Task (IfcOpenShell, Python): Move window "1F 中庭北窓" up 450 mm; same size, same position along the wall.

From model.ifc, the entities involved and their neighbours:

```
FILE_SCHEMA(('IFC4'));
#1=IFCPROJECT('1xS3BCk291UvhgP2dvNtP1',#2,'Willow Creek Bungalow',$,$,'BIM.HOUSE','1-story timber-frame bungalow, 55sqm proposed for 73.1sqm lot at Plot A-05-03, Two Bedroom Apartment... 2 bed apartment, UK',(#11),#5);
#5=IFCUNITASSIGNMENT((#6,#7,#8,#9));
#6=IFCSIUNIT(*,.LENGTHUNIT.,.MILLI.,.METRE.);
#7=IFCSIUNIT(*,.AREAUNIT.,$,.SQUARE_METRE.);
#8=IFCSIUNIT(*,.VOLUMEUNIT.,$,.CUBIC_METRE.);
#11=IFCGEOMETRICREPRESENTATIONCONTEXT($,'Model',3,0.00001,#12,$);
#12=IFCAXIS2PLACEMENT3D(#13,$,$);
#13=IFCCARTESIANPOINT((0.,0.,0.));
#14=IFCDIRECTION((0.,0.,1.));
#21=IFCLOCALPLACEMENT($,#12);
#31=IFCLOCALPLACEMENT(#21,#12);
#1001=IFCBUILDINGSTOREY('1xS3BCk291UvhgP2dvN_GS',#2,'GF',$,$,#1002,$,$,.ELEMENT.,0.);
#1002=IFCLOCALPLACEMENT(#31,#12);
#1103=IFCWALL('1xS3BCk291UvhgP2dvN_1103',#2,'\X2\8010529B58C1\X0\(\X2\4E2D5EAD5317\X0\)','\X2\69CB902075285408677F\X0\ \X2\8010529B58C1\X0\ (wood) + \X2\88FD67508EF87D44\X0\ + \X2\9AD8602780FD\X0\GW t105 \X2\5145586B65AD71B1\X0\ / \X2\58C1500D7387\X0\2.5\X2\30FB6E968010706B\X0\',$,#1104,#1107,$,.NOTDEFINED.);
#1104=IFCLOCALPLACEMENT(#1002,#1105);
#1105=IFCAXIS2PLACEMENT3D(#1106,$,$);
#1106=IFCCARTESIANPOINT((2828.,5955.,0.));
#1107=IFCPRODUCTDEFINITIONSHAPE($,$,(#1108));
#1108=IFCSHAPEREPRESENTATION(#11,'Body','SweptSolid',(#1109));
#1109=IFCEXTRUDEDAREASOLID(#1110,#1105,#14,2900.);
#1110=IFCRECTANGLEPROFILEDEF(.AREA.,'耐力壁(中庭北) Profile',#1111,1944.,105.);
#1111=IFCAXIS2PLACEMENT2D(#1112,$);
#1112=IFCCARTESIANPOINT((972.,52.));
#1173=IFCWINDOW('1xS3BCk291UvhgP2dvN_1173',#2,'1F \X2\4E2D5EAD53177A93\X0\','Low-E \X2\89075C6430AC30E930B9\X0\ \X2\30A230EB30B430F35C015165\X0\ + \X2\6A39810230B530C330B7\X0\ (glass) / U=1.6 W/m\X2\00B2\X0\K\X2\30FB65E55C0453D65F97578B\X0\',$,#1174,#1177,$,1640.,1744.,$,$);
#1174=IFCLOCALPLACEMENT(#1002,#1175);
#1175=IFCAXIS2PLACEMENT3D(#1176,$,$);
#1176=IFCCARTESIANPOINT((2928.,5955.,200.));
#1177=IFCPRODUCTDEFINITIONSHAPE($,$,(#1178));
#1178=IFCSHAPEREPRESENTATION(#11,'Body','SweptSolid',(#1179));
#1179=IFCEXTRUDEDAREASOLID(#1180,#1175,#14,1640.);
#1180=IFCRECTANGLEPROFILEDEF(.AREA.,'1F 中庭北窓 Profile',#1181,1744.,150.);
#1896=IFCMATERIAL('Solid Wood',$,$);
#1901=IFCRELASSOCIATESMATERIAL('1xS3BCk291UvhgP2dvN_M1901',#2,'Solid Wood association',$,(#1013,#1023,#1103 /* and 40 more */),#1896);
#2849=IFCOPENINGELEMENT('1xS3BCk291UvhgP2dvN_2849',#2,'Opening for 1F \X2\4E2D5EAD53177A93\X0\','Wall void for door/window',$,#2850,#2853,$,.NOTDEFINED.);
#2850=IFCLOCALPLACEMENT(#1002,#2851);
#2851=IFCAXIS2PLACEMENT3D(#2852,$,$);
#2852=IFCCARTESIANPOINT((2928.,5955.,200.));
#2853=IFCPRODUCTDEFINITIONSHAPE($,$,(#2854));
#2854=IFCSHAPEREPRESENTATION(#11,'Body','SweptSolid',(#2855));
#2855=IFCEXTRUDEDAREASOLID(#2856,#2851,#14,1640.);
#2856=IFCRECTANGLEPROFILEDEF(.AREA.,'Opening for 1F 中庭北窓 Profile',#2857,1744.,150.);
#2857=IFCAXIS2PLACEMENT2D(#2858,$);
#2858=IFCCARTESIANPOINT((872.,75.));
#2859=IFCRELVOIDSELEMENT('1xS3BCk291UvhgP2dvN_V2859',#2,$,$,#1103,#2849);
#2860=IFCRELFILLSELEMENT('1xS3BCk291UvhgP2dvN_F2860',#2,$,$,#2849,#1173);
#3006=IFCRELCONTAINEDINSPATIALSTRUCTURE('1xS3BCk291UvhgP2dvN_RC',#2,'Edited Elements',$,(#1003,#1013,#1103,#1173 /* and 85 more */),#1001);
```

```python
import numpy as np
import ifcopenshell
import ifcopenshell.api.geometry
import ifcopenshell.util.placement
import ifcopenshell.util.unit

model = ifcopenshell.open("model.ifc")
unit_scale = ifcopenshell.util.unit.calculate_unit_scale(model)

window = model.by_guid("1xS3BCk291UvhgP2dvN_1173")
opening = window.FillsVoids[0].RelatingOpeningElement
dz = 0.45 / unit_scale

shift = np.array([0.0, 0.0, dz])
# The window is not placed relative to its opening, so move both.
for product in (opening, window):
    matrix = ifcopenshell.util.placement.get_local_placement(product.ObjectPlacement)
    matrix[:3, 3] += shift
    ifcopenshell.api.geometry.edit_object_placement(model, product=product, matrix=matrix, is_si=False)

print(f"moved by {dz * unit_scale:+.3f} m")

model.write("model_rev.ifc")
```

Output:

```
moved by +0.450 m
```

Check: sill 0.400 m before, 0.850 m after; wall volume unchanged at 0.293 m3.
